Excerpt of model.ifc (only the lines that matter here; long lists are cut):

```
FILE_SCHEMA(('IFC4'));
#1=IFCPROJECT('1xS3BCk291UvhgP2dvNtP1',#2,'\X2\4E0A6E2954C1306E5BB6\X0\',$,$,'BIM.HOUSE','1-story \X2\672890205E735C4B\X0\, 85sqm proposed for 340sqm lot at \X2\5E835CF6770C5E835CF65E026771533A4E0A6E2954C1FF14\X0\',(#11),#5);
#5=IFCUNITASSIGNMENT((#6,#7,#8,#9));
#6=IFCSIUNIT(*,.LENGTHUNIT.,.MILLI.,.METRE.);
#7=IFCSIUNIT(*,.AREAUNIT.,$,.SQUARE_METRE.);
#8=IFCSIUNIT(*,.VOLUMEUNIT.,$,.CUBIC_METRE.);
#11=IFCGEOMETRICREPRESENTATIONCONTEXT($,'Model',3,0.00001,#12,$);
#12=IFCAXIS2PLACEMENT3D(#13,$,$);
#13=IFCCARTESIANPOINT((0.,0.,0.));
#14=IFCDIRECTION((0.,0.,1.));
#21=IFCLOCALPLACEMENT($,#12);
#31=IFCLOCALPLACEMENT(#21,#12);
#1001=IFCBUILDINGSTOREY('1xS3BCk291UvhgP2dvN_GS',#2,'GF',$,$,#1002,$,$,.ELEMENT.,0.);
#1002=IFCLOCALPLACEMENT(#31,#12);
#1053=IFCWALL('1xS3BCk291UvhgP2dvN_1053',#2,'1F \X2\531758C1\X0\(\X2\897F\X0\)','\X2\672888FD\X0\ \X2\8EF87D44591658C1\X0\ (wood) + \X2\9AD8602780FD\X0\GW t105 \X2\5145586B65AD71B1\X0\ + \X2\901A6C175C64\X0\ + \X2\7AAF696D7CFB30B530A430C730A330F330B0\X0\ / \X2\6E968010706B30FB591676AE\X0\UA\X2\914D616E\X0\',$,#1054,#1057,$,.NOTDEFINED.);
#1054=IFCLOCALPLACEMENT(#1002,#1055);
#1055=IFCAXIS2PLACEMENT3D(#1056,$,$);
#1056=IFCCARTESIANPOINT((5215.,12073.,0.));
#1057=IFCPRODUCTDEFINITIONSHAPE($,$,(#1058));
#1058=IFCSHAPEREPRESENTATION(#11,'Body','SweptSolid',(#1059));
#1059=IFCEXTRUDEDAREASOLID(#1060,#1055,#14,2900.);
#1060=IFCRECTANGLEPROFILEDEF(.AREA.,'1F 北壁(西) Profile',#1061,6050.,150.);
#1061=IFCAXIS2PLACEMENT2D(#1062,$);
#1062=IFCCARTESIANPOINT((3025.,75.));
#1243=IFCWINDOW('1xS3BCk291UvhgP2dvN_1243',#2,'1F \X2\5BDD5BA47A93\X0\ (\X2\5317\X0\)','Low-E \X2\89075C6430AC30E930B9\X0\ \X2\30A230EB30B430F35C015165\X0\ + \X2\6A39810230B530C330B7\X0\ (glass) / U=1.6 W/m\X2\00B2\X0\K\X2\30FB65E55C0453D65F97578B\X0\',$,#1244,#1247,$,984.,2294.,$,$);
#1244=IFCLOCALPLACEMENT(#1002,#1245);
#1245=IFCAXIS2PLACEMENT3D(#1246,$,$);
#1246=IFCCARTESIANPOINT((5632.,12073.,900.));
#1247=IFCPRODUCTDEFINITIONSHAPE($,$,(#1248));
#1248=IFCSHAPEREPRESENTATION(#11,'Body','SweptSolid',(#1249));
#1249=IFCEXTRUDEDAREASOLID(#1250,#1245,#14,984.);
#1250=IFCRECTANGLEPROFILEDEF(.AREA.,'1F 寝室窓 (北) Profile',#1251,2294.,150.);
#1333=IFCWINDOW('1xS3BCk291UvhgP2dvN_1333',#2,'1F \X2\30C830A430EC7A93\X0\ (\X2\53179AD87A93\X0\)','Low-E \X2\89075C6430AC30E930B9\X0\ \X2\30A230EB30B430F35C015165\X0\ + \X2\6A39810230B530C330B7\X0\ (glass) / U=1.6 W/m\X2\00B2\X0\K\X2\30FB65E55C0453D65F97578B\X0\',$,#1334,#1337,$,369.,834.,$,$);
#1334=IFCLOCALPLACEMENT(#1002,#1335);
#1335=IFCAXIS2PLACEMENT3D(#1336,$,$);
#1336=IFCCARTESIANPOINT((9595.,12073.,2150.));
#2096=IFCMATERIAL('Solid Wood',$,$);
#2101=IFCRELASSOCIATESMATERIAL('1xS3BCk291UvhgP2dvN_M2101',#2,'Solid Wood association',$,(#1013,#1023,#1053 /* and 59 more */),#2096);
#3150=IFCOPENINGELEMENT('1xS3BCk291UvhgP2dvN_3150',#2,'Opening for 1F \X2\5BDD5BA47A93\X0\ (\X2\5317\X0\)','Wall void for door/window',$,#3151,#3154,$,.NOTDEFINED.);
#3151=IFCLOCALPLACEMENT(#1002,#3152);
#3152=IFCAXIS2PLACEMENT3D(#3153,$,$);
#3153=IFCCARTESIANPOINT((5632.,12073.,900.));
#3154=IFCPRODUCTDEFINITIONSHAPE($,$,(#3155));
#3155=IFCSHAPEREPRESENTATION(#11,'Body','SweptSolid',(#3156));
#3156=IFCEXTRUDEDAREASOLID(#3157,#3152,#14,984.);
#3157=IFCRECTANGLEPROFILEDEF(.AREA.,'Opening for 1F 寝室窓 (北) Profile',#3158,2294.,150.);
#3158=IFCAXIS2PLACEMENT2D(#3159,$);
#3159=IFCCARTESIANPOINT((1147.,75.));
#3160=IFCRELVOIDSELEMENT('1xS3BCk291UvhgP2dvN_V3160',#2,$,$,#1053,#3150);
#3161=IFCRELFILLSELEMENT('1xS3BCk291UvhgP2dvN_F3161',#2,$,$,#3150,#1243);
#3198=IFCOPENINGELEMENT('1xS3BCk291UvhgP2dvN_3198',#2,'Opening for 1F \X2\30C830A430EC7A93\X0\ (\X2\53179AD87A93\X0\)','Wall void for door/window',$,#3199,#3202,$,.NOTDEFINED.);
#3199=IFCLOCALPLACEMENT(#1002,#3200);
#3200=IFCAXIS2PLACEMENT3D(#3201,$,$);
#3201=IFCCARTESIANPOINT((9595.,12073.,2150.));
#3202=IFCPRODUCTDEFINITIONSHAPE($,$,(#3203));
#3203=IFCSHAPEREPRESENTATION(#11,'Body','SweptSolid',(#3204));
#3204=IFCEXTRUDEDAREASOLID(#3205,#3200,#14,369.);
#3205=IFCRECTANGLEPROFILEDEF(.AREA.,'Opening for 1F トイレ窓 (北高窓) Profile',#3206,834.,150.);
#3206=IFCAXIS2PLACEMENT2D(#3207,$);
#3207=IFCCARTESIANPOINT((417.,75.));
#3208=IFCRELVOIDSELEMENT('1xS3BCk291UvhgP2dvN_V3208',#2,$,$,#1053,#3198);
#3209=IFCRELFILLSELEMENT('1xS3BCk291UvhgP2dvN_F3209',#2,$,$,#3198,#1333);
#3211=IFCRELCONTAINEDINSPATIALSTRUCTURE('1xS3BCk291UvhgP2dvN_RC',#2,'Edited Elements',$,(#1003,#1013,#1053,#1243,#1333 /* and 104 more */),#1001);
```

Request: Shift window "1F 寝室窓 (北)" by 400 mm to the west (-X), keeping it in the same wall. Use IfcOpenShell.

```python
import ifcopenshell
import ifcopenshell.api.geometry
import ifcopenshell.util.placement
import ifcopenshell.util.unit

model = ifcopenshell.open("model.ifc")
unit_scale = ifcopenshell.util.unit.calculate_unit_scale(model)

window = model.by_guid("1xS3BCk291UvhgP2dvN_1243")
opening = window.FillsVoids[0].RelatingOpeningElement
wall = opening.VoidsElements[0].RelatingBuildingElement

wall_matrix = ifcopenshell.util.placement.get_local_placement(wall.ObjectPlacement)
shift = wall_matrix[:3, 0] * -0.4 / unit_scale
before = ifcopenshell.util.placement.get_local_placement(window.ObjectPlacement)[:3, 3].copy()

# The window is not placed relative to its opening, so move both.
for product in (opening, window):
    matrix = ifcopenshell.util.placement.get_local_placement(product.ObjectPlacement)
    matrix[:3, 3] += shift
    ifcopenshell.api.geometry.edit_object_placement(model, product=product, matrix=matrix, is_si=False)

after = ifcopenshell.util.placement.get_local_placement(window.ObjectPlacement)[:3, 3]
print("window moved by", (after - before).round(3) + 0.0)

model.write("model_rev.ifc")
```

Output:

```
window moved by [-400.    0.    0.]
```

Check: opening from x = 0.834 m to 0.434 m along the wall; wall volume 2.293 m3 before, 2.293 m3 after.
